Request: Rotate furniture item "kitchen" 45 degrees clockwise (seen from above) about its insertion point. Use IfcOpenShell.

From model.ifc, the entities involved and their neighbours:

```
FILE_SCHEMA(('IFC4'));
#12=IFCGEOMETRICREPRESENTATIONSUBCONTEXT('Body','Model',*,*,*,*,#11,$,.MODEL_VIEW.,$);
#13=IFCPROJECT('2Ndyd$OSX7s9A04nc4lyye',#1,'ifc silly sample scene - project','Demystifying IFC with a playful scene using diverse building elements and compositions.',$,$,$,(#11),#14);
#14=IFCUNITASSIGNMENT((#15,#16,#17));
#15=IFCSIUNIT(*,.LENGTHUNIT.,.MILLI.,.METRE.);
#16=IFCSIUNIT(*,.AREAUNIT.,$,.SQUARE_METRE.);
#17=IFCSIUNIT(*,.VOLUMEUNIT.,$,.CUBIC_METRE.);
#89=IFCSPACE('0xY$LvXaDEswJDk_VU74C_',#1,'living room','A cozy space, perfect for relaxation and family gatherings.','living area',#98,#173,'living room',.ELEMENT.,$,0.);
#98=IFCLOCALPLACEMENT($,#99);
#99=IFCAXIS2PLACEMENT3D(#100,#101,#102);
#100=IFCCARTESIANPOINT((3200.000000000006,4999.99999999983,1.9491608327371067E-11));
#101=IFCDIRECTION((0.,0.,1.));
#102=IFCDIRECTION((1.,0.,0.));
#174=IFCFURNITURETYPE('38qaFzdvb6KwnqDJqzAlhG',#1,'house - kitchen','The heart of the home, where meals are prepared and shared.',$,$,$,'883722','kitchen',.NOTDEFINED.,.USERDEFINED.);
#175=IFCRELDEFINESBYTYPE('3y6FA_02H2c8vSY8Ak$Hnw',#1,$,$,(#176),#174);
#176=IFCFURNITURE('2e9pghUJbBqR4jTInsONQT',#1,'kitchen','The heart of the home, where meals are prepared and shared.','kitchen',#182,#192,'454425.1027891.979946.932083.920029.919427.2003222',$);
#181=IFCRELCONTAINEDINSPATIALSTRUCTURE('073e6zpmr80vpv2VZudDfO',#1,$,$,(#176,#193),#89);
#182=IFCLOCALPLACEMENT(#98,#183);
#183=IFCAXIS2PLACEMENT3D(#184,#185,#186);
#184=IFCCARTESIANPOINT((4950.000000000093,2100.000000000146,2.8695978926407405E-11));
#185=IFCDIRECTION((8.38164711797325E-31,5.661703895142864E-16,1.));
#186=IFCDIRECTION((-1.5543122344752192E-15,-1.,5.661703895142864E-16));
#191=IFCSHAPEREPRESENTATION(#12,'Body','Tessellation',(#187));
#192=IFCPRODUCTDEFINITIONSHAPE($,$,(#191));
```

```python
import ifcopenshell
import ifcopenshell.api.geometry
import ifcopenshell.util.placement

model = ifcopenshell.open("model.ifc")

item = model.by_guid("2e9pghUJbBqR4jTInsONQT")
matrix = ifcopenshell.util.placement.get_local_placement(item.ObjectPlacement)
matrix = matrix @ ifcopenshell.util.placement.rotation(-45, "Z")
ifcopenshell.api.geometry.edit_object_placement(model, product=item, matrix=matrix, is_si=False)

print(ifcopenshell.util.placement.get_local_placement(item.ObjectPlacement).round(3) + 0.0)

model.write("model-out.ifc")
```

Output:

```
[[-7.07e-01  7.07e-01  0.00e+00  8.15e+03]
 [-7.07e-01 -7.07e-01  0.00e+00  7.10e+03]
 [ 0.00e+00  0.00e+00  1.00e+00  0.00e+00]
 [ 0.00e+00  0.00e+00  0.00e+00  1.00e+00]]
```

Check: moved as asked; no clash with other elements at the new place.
